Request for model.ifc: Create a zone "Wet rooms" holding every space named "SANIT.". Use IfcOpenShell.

First a look at what the model holds.

```python
import ifcopenshell

model = ifcopenshell.open("model.ifc")
print(model.schema)
seen = {}
for space in model.by_type("IfcSpace"):
    seen[space.LongName] = seen.get(space.LongName, 0) + 1
for name, count in sorted(seen.items(), key=str):
    print(count, "x", name)
print("zones:", [z.Name for z in model.by_type("IfcZone")][:20])
```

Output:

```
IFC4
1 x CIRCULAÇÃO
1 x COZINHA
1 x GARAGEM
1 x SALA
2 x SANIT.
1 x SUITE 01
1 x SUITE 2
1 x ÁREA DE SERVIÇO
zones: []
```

```python
import ifcopenshell
import ifcopenshell.api.group
import ifcopenshell.api.root

model = ifcopenshell.open("model.ifc")

names = {"SANIT."}
spaces = [s for s in model.by_type("IfcSpace") if s.LongName in names]

zone = ifcopenshell.api.root.create_entity(model, ifc_class="IfcZone", name="Wet rooms")
ifcopenshell.api.group.assign_group(model, products=spaces, group=zone)
print(len(spaces), "spaces in", zone.Name)

model.write("model_updated.ifc")
```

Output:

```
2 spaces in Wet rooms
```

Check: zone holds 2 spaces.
